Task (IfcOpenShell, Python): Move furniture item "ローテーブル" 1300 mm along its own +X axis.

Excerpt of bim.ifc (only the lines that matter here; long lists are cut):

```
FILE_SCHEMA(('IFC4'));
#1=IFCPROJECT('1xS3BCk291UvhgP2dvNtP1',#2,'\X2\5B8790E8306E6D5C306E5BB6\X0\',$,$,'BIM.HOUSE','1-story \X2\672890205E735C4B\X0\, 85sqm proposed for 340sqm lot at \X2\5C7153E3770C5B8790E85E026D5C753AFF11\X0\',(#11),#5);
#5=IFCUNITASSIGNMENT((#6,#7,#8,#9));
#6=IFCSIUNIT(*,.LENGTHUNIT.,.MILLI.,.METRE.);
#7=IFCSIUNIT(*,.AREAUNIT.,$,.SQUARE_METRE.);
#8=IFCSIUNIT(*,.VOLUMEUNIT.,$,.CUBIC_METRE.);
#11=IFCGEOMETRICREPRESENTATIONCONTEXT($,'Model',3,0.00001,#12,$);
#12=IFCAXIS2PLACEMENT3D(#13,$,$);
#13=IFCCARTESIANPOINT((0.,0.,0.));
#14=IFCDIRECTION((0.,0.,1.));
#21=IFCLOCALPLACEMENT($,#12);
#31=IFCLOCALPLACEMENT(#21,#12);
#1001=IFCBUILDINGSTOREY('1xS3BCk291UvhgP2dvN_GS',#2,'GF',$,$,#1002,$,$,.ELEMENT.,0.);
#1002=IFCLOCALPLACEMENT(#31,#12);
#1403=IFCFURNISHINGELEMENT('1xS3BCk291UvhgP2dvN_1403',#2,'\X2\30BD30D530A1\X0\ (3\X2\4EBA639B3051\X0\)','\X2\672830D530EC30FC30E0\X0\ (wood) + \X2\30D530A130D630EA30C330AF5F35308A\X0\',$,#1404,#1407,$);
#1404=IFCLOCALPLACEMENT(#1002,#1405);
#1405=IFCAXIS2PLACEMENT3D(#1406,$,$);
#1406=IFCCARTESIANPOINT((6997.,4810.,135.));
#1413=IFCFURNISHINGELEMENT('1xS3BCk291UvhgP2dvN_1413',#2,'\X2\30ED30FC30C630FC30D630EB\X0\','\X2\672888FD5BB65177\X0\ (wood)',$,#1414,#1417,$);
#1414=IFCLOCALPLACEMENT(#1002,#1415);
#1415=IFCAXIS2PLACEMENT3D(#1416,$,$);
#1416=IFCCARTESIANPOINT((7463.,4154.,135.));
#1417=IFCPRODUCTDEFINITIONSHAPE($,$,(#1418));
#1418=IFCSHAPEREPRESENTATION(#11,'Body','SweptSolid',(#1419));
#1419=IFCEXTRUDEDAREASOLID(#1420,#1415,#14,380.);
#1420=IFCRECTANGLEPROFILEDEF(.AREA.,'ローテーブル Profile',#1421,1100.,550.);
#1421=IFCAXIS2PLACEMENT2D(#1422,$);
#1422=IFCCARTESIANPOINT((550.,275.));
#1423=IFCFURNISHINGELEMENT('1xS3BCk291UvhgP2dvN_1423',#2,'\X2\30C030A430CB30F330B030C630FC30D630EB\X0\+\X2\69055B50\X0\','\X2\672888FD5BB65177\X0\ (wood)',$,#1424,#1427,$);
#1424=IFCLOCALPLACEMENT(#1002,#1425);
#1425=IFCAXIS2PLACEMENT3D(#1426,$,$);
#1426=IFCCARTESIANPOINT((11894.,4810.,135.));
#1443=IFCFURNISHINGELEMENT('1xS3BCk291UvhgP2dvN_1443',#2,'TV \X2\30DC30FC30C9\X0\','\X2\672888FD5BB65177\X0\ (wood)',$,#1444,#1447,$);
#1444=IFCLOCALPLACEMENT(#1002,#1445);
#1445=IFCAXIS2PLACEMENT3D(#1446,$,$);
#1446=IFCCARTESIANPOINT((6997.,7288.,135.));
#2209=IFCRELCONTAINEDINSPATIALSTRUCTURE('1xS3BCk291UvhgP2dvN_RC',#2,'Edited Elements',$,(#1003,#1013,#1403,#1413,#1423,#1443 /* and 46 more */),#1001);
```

```python
import ifcopenshell
import ifcopenshell.api.geometry
import ifcopenshell.util.placement
import ifcopenshell.util.unit

model = ifcopenshell.open("bim.ifc")
unit_scale = ifcopenshell.util.unit.calculate_unit_scale(model)

item = model.by_guid("1xS3BCk291UvhgP2dvN_1413")
matrix = ifcopenshell.util.placement.get_local_placement(item.ObjectPlacement)
matrix[:3, 3] += matrix[:3, 0] * 1.3 / unit_scale
ifcopenshell.api.geometry.edit_object_placement(model, product=item, matrix=matrix, is_si=False)

print(ifcopenshell.util.placement.get_local_placement(item.ObjectPlacement).round(3) + 0.0)

model.write("bim_v2.ifc")
```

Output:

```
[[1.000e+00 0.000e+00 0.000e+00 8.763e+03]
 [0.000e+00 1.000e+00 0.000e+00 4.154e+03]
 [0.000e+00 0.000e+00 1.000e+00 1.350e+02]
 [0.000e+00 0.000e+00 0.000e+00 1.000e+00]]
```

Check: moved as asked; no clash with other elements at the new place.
